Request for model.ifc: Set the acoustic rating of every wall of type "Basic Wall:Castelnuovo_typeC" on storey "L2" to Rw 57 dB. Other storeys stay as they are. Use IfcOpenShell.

First a look at what the model holds.

```python
import ifcopenshell
import ifcopenshell.util.element

model = ifcopenshell.open("model.ifc")
print(model.schema)
storey = next(s for s in model.by_type("IfcBuildingStorey") if s.Name == "L2")
walls = [e for e in ifcopenshell.util.element.get_decomposition(storey) if e.is_a("IfcWall")]
seen = {}
for e in walls:
    element_type = ifcopenshell.util.element.get_type(e)
    key = (element_type.Name if element_type != e and element_type else None, ifcopenshell.util.element.get_pset(e, "Pset_WallCommon", "AcousticRating"))
    seen[key] = seen.get(key, 0) + 1
for (name, value), count in sorted(seen.items(), key=str):
    print(count, "x", name, "|", value)
```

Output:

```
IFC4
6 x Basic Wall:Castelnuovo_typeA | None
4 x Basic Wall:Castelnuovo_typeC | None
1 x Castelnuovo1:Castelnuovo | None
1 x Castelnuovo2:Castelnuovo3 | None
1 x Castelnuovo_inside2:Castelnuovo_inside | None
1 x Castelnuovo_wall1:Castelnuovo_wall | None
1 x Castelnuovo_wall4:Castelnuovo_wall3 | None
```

```python
import ifcopenshell
import ifcopenshell.api.pset
import ifcopenshell.util.element

model = ifcopenshell.open("model.ifc")

storey = next(s for s in model.by_type("IfcBuildingStorey") if s.Name == "L2")
walls = [e for e in ifcopenshell.util.element.get_decomposition(storey) if e.is_a("IfcWall")]

count = 0
for e in walls:
    element_type = ifcopenshell.util.element.get_type(e)
    if element_type in (None, e) or element_type.Name != "Basic Wall:Castelnuovo_typeC":
        continue
    # add_pset returns the element's existing set when there is one.
    pset = ifcopenshell.api.pset.add_pset(model, product=e, name="Pset_WallCommon")
    ifcopenshell.api.pset.edit_pset(model, pset=pset, properties={"AcousticRating": "Rw 57 dB"})
    count += 1

print(count, "walls updated")

model.write("model-out.ifc")
```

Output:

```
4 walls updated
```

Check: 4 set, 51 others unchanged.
